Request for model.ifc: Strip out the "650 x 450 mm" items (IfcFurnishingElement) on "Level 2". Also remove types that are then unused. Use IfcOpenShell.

First a look at what the model holds.

```python
import ifcopenshell
import ifcopenshell.util.element

model = ifcopenshell.open("model.ifc")
print(model.schema)
storey = next(s for s in model.by_type("IfcBuildingStorey") if s.Name == "Level 2")
furniture = [e for e in ifcopenshell.util.element.get_decomposition(storey) if e.is_a("IfcFurnishingElement")]
seen = {}
for e in furniture:
    element_type = ifcopenshell.util.element.get_type(e)
    name = element_type.Name if element_type not in (None, e) else None
    seen[name] = seen.get(name, 0) + 1
for name, count in sorted(seen.items(), key=str):
    print(count, "x", name)
```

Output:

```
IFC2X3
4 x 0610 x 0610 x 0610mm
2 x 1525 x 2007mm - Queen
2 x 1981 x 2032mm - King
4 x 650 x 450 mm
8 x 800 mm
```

```python
import ifcopenshell
import ifcopenshell.api.root
import ifcopenshell.util.element

model = ifcopenshell.open("model.ifc")

storey = next(s for s in model.by_type("IfcBuildingStorey") if s.Name == "Level 2")
furniture = [e for e in ifcopenshell.util.element.get_decomposition(storey) if e.is_a("IfcFurnishingElement")]
targets = [e for e in furniture if (t := ifcopenshell.util.element.get_type(e)) not in (None, e) and t.Name == "650 x 450 mm"]
types = {ifcopenshell.util.element.get_type(e) for e in targets} - {None, *targets}

for e in targets:
    ifcopenshell.api.root.remove_product(model, product=e)
print(len(targets), "removed")

unused = [t for t in types if not ifcopenshell.util.element.get_types(t)]
for t in unused:
    ifcopenshell.api.root.remove_product(model, product=t)
print(len(unused), "unused types removed")

model.write("model_updated.ifc")
```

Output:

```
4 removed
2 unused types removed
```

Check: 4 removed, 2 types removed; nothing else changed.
